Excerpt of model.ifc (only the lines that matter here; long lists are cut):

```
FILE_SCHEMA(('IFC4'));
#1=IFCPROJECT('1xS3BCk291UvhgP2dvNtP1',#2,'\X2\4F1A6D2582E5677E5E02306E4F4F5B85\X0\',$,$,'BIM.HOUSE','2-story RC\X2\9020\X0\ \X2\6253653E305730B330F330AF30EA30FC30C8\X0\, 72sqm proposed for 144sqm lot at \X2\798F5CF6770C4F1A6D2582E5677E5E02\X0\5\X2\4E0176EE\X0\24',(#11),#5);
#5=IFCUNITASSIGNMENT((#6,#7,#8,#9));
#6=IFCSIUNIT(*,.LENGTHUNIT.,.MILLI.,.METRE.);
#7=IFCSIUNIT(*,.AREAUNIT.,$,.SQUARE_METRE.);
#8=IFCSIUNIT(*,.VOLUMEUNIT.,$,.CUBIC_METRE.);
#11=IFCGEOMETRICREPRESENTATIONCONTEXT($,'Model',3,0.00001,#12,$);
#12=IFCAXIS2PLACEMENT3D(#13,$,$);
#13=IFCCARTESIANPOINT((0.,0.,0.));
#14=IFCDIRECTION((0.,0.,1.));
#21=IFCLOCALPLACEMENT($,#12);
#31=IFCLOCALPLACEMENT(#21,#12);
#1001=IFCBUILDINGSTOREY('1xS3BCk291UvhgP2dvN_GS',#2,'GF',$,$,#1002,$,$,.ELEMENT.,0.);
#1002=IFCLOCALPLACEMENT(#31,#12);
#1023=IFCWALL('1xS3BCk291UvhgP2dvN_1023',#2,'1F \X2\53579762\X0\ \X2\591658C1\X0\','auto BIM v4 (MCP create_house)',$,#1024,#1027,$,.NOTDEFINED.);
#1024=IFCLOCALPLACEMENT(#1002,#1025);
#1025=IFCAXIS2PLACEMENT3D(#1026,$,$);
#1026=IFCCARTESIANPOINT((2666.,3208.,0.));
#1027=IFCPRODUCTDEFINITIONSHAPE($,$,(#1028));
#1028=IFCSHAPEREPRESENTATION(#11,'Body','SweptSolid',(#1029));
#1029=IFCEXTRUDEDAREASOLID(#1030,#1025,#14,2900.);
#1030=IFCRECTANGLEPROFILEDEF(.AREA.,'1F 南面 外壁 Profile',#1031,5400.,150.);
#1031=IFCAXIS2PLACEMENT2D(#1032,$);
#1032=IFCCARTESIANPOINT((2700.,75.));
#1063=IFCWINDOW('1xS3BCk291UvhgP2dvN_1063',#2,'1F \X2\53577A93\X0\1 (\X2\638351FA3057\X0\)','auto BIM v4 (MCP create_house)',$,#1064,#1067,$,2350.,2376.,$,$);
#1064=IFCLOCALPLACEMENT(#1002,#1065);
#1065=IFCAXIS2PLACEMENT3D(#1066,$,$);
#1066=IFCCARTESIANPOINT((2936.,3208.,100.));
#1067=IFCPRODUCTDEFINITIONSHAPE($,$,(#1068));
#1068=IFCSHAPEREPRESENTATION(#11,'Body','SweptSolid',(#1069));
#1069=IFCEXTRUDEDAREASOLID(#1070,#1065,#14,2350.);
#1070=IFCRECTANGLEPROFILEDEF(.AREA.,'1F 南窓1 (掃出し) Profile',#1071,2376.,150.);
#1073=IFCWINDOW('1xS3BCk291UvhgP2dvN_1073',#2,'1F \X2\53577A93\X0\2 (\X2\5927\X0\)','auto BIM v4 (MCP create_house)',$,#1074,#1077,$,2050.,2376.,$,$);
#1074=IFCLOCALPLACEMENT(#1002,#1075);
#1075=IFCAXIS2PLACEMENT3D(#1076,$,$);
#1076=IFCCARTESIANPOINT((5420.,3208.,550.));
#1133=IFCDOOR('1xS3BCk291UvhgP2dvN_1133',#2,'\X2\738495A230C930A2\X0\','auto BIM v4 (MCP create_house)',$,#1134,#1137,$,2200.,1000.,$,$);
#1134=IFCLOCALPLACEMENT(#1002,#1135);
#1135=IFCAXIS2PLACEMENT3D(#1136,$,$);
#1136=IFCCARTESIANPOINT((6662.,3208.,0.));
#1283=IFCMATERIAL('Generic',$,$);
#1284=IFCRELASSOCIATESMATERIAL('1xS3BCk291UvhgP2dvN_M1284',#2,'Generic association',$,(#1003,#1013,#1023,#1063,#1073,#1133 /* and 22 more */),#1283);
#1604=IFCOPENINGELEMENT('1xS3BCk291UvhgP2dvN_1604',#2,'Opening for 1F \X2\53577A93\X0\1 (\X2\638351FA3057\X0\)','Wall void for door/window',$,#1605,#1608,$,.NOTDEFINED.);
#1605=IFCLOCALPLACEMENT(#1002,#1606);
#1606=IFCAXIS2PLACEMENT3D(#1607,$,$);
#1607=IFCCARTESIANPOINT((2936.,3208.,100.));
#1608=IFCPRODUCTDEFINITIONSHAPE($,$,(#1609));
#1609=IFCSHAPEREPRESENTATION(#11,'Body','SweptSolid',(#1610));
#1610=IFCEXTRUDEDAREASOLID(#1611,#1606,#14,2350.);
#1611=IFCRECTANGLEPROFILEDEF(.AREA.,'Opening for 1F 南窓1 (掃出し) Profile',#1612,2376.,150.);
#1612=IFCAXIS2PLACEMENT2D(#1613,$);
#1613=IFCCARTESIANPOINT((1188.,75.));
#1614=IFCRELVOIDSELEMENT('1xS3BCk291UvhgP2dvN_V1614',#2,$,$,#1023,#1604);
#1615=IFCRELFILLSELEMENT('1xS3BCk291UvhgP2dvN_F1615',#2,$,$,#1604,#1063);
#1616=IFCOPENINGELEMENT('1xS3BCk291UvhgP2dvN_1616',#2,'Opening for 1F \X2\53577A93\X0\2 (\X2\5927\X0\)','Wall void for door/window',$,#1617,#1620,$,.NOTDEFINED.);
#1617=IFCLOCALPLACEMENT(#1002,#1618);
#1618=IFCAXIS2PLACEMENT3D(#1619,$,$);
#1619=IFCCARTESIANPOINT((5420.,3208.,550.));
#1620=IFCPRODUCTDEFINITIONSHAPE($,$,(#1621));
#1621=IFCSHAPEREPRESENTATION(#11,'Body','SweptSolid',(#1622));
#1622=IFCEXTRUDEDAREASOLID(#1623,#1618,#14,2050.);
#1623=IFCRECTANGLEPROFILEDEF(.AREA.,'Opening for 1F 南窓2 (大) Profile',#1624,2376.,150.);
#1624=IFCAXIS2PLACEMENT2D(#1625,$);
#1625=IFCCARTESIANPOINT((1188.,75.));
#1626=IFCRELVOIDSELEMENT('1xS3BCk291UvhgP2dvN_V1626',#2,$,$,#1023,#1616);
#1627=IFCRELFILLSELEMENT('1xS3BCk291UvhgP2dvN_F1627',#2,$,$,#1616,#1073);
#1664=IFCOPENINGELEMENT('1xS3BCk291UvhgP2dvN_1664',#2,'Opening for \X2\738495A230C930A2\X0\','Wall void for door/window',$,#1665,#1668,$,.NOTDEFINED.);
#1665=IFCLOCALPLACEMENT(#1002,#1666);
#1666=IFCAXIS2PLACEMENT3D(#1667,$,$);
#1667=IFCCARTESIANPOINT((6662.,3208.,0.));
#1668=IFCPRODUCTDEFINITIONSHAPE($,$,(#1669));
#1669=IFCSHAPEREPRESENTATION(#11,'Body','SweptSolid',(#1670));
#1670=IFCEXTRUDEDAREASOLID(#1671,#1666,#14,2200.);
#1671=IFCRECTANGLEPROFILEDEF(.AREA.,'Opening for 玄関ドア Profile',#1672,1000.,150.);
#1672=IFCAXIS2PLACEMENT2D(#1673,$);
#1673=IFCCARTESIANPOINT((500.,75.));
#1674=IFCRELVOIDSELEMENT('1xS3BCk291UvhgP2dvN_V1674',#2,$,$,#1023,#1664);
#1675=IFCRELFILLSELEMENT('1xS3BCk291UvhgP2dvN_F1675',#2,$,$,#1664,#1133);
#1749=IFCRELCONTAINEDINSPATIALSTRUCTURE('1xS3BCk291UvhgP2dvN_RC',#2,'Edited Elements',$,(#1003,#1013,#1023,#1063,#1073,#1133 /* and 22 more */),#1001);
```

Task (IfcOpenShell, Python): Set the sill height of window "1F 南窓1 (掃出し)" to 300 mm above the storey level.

```python
import numpy as np
import ifcopenshell
import ifcopenshell.api.geometry
import ifcopenshell.geom
import ifcopenshell.util.element
import ifcopenshell.util.placement
import ifcopenshell.util.shape
import ifcopenshell.util.unit

model = ifcopenshell.open("model.ifc")
unit_scale = ifcopenshell.util.unit.calculate_unit_scale(model)

window = model.by_id(1063)
opening = window.FillsVoids[0].RelatingOpeningElement
storey = ifcopenshell.util.element.get_container(window, ifc_class="IfcBuildingStorey")
level = ifcopenshell.util.placement.get_local_placement(storey.ObjectPlacement)[2, 3]

# The opening's origin need not be at the sill, so measure its lowest point.
shape = ifcopenshell.geom.create_shape(ifcopenshell.geom.settings(), opening)
bottom = ifcopenshell.util.shape.get_shape_bottom_elevation(shape, shape.geometry) / unit_scale
dz = level + 0.3 / unit_scale - bottom

shift = np.array([0.0, 0.0, dz])
# The window is not placed relative to its opening, so move both.
for product in (opening, window):
    matrix = ifcopenshell.util.placement.get_local_placement(product.ObjectPlacement)
    matrix[:3, 3] += shift
    ifcopenshell.api.geometry.edit_object_placement(model, product=product, matrix=matrix, is_si=False)

print(f"moved by {dz * unit_scale:+.3f} m")

model.write("model_edited.ifc")
```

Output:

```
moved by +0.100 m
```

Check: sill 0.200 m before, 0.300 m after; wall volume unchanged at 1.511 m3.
